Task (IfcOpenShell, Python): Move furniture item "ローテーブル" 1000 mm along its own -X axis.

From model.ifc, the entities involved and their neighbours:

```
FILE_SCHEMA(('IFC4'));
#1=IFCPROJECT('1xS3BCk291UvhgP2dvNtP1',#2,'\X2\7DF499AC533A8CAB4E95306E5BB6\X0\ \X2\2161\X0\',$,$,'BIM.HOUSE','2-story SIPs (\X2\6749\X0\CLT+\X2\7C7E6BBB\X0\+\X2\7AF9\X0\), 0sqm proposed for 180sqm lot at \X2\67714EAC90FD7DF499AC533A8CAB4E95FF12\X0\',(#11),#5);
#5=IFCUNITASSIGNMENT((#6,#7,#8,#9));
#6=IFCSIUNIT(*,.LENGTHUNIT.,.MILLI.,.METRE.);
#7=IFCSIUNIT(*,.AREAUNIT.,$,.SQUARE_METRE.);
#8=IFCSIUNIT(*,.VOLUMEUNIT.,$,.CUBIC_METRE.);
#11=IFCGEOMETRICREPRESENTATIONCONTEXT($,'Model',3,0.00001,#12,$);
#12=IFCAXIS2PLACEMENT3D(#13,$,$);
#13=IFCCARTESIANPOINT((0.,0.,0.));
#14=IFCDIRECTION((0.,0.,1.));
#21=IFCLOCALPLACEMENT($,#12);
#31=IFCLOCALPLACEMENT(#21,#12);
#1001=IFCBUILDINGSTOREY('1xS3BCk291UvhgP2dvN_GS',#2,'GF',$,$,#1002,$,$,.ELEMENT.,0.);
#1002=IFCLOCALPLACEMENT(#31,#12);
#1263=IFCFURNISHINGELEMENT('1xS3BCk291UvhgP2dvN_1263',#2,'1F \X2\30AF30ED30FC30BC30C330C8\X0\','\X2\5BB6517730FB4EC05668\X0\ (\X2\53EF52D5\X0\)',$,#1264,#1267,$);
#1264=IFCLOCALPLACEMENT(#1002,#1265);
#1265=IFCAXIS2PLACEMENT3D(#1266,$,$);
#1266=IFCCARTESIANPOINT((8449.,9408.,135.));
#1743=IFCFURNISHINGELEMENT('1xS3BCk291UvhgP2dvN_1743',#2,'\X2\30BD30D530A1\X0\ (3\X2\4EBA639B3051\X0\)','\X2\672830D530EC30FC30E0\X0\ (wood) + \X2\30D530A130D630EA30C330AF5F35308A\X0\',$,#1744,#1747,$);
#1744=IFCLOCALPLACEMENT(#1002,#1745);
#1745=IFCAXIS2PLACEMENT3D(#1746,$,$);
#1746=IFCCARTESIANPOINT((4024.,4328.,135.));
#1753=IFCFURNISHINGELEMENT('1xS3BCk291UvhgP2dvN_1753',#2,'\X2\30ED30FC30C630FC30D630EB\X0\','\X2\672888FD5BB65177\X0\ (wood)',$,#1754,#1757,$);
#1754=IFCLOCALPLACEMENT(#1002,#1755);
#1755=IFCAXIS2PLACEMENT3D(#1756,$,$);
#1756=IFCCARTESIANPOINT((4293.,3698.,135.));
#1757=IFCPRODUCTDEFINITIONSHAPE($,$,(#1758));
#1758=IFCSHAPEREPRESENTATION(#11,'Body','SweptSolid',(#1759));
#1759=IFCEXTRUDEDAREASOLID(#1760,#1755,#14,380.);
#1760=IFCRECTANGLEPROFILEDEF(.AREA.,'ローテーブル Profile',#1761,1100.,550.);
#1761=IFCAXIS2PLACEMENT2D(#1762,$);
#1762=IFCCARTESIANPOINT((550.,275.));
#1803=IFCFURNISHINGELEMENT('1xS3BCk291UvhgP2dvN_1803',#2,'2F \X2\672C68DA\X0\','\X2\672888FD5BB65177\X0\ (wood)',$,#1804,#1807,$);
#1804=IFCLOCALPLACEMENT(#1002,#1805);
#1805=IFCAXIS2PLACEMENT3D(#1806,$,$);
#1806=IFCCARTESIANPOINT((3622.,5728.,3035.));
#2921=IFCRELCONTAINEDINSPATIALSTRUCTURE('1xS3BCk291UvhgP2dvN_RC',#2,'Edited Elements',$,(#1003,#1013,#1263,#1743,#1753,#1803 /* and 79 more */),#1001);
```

```python
import ifcopenshell
import ifcopenshell.api.geometry
import ifcopenshell.util.placement

model = ifcopenshell.open("model.ifc")

item = model.by_guid("1xS3BCk291UvhgP2dvN_1753")
matrix = ifcopenshell.util.placement.get_local_placement(item.ObjectPlacement)
matrix[:3, 3] -= matrix[:3, 0] * 1000.0
ifcopenshell.api.geometry.edit_object_placement(model, product=item, matrix=matrix, is_si=False)

print(ifcopenshell.util.placement.get_local_placement(item.ObjectPlacement).round(3) + 0.0)

model.write("model_rev.ifc")
```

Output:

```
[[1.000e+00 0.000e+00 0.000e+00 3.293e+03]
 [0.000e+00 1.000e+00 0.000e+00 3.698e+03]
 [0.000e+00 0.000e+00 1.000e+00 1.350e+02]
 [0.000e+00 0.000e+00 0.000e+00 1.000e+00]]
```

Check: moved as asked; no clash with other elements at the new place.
